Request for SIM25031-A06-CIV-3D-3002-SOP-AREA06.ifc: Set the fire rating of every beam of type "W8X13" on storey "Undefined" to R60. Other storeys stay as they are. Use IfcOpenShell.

First a look at what the model holds.

```python
import ifcopenshell
import ifcopenshell.util.element

model = ifcopenshell.open("SIM25031-A06-CIV-3D-3002-SOP-AREA06.ifc")
print(model.schema)
storey = next(s for s in model.by_type("IfcBuildingStorey") if s.Name == "Undefined")
beams = [e for e in ifcopenshell.util.element.get_decomposition(storey) if e.is_a("IfcBeam")]
seen = {}
for e in beams:
    element_type = ifcopenshell.util.element.get_type(e)
    key = (element_type.Name if element_type != e and element_type else None, ifcopenshell.util.element.get_pset(e, "Pset_BeamCommon", "FireRating"))
    seen[key] = seen.get(key, 0) + 1
for (name, value), count in sorted(seen.items(), key=str):
    print(count, "x", name, "|", value)
```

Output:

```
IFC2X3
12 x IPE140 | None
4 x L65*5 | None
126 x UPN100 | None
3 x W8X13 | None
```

```python
import ifcopenshell
import ifcopenshell.api.pset
import ifcopenshell.util.element

model = ifcopenshell.open("SIM25031-A06-CIV-3D-3002-SOP-AREA06.ifc")

storey = next(s for s in model.by_type("IfcBuildingStorey") if s.Name == "Undefined")
beams = [e for e in ifcopenshell.util.element.get_decomposition(storey) if e.is_a("IfcBeam")]

count = 0
for e in beams:
    element_type = ifcopenshell.util.element.get_type(e)
    if element_type in (None, e) or element_type.Name != "W8X13":
        continue
    found = ifcopenshell.util.element.get_pset(e, "Pset_BeamCommon", should_inherit=False)
    if found:
        pset = model.by_id(found["id"])
        if len(ifcopenshell.util.element.get_elements_by_pset(pset)) > 1:
            pset = ifcopenshell.api.pset.unshare_pset(model, products=[e], pset=pset)[0]
    else:
        pset = ifcopenshell.api.pset.add_pset(model, product=e, name="Pset_BeamCommon")
    ifcopenshell.api.pset.edit_pset(model, pset=pset, properties={"FireRating": "R60"})
    count += 1

print(count, "beams updated")

model.write("SIM25031-A06-CIV-3D-3002-SOP-AREA06-out.ifc")
```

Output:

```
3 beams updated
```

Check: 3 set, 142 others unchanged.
